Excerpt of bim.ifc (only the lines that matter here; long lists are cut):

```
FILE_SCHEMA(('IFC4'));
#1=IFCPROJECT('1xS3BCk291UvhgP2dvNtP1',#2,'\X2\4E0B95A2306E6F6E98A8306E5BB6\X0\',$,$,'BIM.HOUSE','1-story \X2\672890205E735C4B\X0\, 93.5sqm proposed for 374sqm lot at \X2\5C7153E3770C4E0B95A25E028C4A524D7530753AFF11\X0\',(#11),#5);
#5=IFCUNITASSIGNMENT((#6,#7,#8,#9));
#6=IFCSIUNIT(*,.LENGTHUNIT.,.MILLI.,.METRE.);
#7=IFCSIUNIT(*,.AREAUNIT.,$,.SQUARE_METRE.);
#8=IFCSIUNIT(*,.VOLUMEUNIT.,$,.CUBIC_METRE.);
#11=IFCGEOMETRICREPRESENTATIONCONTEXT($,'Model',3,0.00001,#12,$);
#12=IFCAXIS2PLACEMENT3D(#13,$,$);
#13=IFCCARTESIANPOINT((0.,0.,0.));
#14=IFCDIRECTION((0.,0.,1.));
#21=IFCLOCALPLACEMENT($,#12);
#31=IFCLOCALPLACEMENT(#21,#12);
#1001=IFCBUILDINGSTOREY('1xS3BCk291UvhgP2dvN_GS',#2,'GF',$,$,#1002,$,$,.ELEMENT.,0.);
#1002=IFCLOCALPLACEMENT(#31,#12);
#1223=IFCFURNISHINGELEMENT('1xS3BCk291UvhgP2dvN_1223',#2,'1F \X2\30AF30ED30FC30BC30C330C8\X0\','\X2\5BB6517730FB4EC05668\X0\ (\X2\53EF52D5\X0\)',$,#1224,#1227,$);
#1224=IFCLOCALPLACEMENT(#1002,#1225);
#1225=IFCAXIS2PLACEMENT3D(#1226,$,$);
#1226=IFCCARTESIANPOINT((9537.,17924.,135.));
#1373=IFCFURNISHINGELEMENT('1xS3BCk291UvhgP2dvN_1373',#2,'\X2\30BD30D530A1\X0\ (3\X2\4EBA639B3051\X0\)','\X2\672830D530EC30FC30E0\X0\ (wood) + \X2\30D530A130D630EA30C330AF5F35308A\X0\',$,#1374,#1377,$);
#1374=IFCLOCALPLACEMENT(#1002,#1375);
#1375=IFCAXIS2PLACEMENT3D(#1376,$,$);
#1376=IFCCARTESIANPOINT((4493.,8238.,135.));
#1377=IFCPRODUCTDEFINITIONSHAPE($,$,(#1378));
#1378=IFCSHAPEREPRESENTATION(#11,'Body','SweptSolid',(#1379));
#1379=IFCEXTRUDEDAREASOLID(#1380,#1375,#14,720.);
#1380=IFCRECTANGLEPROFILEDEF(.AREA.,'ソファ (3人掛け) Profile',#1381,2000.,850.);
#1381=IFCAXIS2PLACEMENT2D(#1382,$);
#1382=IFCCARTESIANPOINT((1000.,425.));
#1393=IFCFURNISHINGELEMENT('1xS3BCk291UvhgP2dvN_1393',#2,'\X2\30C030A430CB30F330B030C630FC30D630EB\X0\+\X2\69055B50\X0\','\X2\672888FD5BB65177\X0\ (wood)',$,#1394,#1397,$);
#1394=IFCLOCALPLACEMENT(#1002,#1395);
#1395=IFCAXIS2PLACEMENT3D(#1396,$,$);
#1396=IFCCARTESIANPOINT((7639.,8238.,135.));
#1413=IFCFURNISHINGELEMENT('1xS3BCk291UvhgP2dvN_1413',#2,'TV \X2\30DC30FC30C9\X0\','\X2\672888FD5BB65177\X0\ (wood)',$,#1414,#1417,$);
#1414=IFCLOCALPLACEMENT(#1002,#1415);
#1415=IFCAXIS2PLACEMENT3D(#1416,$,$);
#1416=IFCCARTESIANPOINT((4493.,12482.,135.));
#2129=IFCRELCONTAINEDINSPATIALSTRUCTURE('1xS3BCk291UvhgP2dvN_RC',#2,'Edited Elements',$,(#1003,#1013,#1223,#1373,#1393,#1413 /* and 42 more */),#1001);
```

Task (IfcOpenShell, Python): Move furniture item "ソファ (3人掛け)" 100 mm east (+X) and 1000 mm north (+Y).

```python
import ifcopenshell
import ifcopenshell.api.geometry
import ifcopenshell.util.placement

model = ifcopenshell.open("bim.ifc")

item = model.by_id(1373)
matrix = ifcopenshell.util.placement.get_local_placement(item.ObjectPlacement)
matrix[0, 3] += 100.0
matrix[1, 3] += 1000.0
ifcopenshell.api.geometry.edit_object_placement(model, product=item, matrix=matrix, is_si=False)

print(ifcopenshell.util.placement.get_local_placement(item.ObjectPlacement).round(3) + 0.0)

model.write("bim_rev.ifc")
```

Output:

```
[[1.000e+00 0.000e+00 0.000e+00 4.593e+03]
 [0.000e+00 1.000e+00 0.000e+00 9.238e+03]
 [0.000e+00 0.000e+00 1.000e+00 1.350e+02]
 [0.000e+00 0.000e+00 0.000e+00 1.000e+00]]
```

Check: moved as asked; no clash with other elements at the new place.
